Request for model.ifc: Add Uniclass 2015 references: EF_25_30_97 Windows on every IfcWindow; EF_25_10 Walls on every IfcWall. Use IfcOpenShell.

First a look at what the model holds.

```python
import ifcopenshell

model = ifcopenshell.open("model.ifc")
print(model.schema)
print("classifications:", [c.Name for c in model.by_type("IfcClassification")])
for ifc_class in ("IfcDoor", "IfcRoof", "IfcStair", "IfcWall", "IfcWindow"):
    print(ifc_class, len(model.by_type(ifc_class)))
```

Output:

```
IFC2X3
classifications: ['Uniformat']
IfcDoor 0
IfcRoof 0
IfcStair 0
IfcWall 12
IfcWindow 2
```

```python
import ifcopenshell
import ifcopenshell.api.classification

model = ifcopenshell.open("model.ifc")

# IFC2X3 requires Source and Edition and has no link from the project to the system.
system = model.create_entity("IfcClassification", Source="NBS", Edition="2015", Name="Uniclass 2015")

codes = {
    "IfcWindow": ("EF_25_30_97", "Windows"),
    "IfcWall": ("EF_25_10", "Walls"),
}
for ifc_class, (code, name) in codes.items():
    products = model.by_type(ifc_class)
    ifcopenshell.api.classification.add_reference(
        model, products=products, classification=system, identification=code, name=name
    )
    print(code, len(products))

model.write("model_rev.ifc")
```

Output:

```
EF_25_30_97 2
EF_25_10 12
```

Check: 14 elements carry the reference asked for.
